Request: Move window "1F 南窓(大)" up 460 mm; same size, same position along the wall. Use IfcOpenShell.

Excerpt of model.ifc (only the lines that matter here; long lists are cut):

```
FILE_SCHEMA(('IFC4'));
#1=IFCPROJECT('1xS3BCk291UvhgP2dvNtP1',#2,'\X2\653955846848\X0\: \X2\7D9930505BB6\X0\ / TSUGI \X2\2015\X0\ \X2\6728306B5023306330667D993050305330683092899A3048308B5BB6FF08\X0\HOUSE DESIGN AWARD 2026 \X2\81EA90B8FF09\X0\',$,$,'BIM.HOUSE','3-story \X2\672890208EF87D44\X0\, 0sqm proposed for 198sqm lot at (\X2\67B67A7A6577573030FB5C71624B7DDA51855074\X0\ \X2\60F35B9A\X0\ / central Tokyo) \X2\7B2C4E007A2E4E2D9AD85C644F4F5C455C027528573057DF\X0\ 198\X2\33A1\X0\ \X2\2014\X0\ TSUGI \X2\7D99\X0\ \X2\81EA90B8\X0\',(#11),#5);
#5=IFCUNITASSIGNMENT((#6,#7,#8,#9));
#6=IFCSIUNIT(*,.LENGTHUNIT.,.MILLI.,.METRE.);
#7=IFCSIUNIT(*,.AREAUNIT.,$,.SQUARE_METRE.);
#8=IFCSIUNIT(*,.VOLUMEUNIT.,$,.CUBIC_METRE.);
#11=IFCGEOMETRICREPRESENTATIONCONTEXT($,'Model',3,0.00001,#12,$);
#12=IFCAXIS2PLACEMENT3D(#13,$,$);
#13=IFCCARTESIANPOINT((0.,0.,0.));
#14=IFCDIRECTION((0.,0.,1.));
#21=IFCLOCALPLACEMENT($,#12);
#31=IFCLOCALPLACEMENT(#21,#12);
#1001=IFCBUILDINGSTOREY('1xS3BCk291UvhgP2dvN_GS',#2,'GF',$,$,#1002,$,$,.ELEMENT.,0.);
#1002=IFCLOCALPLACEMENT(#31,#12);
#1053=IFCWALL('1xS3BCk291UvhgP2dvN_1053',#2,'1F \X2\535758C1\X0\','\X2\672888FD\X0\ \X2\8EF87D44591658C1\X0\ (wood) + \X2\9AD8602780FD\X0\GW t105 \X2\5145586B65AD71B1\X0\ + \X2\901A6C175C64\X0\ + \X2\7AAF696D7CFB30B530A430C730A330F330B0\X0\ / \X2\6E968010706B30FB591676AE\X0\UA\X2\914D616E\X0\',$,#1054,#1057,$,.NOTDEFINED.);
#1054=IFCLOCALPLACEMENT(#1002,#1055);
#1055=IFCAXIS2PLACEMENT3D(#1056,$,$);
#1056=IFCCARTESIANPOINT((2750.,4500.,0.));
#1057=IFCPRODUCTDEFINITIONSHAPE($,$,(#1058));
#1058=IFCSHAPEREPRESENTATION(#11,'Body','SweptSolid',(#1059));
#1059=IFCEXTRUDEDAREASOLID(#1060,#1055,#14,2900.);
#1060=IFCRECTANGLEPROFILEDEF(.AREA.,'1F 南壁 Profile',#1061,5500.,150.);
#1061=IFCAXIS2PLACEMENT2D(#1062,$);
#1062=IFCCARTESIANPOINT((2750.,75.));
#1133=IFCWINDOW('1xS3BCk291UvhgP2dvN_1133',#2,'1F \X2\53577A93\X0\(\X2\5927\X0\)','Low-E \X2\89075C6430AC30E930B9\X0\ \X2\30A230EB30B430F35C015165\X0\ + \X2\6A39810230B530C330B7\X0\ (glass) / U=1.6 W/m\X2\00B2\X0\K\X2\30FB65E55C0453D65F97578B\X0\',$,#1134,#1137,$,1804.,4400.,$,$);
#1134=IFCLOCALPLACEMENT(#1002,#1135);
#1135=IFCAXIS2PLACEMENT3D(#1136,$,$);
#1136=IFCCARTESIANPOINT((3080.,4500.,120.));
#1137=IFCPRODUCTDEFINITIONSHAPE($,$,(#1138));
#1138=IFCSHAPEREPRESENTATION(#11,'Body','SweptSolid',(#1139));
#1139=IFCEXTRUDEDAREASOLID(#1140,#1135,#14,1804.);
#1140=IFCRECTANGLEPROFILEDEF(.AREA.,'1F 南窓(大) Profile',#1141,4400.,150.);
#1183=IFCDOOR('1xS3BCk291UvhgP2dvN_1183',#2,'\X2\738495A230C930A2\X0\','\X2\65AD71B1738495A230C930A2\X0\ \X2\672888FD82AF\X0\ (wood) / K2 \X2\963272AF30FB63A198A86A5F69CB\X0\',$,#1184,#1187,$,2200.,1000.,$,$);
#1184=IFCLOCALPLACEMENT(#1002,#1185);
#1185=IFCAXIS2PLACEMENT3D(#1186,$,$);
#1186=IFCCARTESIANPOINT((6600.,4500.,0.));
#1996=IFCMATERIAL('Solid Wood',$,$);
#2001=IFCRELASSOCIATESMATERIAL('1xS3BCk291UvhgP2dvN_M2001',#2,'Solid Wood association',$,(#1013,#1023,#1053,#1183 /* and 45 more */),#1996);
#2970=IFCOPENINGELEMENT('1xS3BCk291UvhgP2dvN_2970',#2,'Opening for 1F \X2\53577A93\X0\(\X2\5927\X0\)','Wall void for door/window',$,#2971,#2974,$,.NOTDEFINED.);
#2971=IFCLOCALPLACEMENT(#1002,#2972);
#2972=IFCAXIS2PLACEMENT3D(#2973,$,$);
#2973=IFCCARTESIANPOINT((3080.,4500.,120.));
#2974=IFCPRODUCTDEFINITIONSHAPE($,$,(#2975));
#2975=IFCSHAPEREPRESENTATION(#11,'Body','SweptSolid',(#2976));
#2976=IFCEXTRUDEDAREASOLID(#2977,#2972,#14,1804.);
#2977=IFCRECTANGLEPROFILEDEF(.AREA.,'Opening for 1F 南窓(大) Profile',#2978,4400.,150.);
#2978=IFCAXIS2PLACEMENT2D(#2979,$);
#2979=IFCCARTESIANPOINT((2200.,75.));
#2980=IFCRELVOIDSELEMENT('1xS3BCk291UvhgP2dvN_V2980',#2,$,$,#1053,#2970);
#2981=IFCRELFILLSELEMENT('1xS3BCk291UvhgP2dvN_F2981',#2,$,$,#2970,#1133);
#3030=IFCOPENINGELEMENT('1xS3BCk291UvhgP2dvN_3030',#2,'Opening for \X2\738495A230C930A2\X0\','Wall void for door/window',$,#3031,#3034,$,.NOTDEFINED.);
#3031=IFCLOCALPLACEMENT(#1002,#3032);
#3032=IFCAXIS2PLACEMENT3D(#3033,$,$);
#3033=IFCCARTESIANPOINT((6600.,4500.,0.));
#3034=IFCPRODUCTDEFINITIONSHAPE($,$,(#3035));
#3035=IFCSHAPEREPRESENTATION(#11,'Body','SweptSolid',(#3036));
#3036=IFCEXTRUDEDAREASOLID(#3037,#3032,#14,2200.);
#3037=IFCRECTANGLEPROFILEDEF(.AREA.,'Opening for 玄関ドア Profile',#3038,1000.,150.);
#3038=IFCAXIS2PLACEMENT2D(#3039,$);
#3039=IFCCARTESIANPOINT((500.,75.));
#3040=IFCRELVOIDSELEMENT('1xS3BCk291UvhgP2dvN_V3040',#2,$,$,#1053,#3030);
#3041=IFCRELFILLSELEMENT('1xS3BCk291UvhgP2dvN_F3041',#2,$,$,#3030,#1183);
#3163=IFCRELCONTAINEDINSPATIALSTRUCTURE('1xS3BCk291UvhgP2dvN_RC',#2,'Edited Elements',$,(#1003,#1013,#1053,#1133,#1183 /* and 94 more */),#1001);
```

```python
import numpy as np
import ifcopenshell
import ifcopenshell.api.geometry
import ifcopenshell.util.placement
import ifcopenshell.util.unit

model = ifcopenshell.open("model.ifc")
unit_scale = ifcopenshell.util.unit.calculate_unit_scale(model)

window = model.by_guid("1xS3BCk291UvhgP2dvN_1133")
opening = window.FillsVoids[0].RelatingOpeningElement
dz = 460.0

shift = np.array([0.0, 0.0, dz])
# The window is not placed relative to its opening, so move both.
for product in (opening, window):
    matrix = ifcopenshell.util.placement.get_local_placement(product.ObjectPlacement)
    matrix[:3, 3] += shift
    ifcopenshell.api.geometry.edit_object_placement(model, product=product, matrix=matrix, is_si=False)

print(f"moved by {dz * unit_scale:+.3f} m")

model.write("model_edited.ifc")
```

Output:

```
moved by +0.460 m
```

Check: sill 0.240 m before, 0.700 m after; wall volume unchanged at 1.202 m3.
